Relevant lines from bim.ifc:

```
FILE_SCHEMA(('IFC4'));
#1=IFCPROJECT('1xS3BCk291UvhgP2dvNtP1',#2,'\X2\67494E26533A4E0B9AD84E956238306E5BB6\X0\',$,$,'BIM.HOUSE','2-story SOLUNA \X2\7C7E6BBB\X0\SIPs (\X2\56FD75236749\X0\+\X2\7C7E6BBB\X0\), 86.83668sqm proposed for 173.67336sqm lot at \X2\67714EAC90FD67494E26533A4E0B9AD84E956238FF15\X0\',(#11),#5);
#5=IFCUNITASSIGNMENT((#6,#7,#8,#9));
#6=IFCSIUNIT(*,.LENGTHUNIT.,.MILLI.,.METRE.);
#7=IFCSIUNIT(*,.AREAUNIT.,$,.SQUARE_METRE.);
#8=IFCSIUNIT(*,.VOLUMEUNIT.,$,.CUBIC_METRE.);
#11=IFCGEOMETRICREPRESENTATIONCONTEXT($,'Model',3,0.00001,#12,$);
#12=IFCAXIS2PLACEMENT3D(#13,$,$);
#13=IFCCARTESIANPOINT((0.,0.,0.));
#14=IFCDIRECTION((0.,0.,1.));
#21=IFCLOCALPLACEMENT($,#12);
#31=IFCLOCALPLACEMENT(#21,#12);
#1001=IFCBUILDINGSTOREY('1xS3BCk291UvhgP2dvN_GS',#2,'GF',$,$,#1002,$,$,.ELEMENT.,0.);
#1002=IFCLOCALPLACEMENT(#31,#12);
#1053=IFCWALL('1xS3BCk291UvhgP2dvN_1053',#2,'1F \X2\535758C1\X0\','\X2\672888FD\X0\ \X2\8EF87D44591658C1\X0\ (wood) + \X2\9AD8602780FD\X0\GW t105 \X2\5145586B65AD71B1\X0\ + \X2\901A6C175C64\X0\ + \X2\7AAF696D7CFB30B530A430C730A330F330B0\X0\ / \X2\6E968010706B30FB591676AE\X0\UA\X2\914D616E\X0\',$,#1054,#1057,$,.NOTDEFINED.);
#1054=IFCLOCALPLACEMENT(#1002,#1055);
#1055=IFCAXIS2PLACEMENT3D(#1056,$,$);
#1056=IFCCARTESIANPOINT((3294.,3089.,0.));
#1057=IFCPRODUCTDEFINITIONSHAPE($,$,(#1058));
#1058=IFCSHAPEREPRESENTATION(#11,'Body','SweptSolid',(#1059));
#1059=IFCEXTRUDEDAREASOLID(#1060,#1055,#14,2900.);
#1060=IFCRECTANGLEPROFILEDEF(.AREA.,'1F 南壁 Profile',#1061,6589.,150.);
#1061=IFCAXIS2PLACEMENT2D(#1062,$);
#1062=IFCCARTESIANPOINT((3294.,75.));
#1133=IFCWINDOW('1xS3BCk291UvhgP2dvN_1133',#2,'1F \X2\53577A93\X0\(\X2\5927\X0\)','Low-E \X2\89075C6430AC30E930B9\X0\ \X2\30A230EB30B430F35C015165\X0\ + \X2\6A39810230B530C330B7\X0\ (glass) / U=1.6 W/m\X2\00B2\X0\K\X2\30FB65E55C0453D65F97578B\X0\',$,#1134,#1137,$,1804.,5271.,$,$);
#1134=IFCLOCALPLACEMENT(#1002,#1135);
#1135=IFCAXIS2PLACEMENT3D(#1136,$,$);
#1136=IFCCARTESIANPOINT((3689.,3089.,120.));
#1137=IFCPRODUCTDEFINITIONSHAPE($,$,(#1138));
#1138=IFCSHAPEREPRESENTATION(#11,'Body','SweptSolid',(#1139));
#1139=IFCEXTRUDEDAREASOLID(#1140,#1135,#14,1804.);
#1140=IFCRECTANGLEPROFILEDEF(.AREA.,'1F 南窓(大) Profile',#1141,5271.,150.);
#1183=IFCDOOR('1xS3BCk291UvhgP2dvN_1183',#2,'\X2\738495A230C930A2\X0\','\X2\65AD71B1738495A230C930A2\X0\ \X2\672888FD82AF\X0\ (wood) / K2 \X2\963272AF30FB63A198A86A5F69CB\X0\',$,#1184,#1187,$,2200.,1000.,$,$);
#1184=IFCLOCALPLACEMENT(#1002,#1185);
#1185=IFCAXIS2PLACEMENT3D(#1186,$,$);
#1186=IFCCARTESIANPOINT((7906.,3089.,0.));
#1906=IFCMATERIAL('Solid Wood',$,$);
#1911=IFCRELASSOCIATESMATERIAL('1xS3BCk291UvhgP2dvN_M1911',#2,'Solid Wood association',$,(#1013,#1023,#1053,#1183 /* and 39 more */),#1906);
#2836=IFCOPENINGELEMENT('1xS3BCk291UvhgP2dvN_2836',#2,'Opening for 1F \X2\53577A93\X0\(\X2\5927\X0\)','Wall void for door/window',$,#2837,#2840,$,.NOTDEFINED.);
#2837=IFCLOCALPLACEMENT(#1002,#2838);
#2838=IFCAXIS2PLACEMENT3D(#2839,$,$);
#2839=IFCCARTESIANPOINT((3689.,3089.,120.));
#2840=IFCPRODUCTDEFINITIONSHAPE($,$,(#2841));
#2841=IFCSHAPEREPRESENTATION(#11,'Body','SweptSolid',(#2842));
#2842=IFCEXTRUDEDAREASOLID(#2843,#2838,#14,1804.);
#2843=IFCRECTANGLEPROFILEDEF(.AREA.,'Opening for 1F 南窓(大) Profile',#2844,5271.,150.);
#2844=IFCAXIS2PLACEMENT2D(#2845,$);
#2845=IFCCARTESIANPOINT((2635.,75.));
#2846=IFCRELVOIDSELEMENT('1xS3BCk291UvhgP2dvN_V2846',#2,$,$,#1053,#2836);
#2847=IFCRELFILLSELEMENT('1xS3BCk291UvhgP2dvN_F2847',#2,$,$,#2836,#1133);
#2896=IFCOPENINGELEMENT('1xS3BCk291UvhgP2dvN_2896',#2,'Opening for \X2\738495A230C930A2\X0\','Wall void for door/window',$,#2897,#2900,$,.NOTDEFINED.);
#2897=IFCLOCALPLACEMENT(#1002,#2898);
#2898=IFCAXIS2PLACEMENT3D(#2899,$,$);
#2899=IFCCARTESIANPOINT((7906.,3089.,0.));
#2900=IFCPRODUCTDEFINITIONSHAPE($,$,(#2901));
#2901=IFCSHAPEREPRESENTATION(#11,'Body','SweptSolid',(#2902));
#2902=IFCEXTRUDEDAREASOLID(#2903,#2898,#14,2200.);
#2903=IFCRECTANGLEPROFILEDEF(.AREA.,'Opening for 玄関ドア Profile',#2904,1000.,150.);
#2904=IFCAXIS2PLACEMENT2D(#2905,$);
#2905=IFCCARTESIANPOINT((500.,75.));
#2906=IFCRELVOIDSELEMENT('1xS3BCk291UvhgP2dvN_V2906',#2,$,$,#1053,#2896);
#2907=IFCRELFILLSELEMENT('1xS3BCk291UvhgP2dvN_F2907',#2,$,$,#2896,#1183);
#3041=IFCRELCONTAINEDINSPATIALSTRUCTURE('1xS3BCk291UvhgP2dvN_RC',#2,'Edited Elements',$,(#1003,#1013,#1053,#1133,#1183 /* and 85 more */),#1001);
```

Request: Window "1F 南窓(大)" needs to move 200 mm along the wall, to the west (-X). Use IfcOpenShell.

```python
import ifcopenshell
import ifcopenshell.api.geometry
import ifcopenshell.util.placement
import ifcopenshell.util.unit

model = ifcopenshell.open("bim.ifc")
unit_scale = ifcopenshell.util.unit.calculate_unit_scale(model)

window = model.by_guid("1xS3BCk291UvhgP2dvN_1133")
opening = window.FillsVoids[0].RelatingOpeningElement
wall = opening.VoidsElements[0].RelatingBuildingElement

wall_matrix = ifcopenshell.util.placement.get_local_placement(wall.ObjectPlacement)
shift = wall_matrix[:3, 0] * -0.2 / unit_scale
before = ifcopenshell.util.placement.get_local_placement(window.ObjectPlacement)[:3, 3].copy()

# The window is not placed relative to its opening, so move both.
for product in (opening, window):
    matrix = ifcopenshell.util.placement.get_local_placement(product.ObjectPlacement)
    matrix[:3, 3] += shift
    ifcopenshell.api.geometry.edit_object_placement(model, product=product, matrix=matrix, is_si=False)

after = ifcopenshell.util.placement.get_local_placement(window.ObjectPlacement)[:3, 3]
print("window moved by", (after - before).round(3) + 0.0)

model.write("bim_updated.ifc")
```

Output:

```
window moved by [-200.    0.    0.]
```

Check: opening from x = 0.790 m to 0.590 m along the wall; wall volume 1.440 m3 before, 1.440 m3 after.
